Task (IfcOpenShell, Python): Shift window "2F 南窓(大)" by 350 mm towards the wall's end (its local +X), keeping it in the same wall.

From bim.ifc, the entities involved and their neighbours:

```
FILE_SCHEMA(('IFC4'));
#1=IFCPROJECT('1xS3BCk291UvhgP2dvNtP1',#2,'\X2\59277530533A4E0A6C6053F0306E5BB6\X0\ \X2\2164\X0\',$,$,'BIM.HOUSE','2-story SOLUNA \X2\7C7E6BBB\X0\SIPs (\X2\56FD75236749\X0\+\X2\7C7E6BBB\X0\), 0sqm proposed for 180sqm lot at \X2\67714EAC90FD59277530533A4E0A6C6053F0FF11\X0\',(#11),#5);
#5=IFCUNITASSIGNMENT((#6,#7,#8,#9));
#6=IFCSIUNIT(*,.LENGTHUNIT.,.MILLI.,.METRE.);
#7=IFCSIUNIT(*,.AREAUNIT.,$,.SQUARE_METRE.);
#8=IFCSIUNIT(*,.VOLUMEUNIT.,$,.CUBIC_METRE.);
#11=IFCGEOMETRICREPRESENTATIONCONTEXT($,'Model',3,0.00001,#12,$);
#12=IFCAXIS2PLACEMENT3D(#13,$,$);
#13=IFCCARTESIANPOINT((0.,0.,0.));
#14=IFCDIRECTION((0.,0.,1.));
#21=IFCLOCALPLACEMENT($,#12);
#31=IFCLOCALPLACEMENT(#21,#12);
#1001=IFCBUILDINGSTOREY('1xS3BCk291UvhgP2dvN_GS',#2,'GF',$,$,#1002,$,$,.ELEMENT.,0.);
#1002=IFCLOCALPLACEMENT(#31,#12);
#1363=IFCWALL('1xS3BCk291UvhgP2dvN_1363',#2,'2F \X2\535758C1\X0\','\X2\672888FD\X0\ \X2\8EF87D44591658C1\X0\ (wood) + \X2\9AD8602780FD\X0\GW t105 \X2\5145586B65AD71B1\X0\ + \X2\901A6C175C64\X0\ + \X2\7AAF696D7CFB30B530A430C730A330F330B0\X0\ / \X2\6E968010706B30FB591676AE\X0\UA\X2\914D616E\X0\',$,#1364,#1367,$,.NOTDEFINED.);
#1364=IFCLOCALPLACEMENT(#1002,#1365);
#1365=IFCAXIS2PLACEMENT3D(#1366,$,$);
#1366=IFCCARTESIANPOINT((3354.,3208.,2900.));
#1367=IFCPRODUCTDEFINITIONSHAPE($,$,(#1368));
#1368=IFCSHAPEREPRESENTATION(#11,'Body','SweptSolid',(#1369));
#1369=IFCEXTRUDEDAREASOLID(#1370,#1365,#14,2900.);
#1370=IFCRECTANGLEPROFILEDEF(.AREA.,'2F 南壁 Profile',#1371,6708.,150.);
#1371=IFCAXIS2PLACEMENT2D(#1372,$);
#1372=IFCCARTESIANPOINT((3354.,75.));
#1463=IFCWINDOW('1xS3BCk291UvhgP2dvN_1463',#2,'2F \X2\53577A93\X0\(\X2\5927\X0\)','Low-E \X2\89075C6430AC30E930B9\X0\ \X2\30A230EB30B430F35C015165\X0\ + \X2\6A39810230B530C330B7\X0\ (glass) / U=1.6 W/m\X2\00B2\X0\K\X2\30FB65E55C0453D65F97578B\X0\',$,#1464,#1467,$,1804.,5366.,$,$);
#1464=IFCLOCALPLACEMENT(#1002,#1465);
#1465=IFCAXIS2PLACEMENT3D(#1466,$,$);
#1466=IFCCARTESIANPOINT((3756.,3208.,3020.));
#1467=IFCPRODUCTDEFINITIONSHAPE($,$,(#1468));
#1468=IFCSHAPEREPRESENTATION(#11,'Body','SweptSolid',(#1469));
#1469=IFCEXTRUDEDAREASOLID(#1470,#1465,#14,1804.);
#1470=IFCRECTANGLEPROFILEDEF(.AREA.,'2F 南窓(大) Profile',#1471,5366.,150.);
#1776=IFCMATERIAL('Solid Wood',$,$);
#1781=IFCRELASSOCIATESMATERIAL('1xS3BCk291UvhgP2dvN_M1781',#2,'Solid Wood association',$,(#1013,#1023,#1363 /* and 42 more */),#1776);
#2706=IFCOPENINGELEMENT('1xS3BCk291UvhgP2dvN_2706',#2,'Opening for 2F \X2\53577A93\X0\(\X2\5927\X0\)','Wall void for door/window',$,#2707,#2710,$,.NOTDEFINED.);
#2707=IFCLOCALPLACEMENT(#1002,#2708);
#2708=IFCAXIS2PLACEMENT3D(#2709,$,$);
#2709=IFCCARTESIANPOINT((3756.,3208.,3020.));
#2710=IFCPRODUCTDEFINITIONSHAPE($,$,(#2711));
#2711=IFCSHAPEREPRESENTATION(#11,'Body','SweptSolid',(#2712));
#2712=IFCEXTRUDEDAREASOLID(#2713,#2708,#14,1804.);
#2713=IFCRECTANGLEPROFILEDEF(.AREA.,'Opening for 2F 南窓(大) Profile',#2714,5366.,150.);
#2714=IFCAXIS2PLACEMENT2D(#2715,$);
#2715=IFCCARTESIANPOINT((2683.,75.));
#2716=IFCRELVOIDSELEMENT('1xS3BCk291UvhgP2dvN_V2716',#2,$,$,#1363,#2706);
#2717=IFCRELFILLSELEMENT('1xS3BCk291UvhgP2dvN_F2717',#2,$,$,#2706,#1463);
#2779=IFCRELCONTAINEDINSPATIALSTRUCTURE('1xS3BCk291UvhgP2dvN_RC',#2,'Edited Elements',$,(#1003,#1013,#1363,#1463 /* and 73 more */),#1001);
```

```python
import ifcopenshell
import ifcopenshell.api.geometry
import ifcopenshell.util.placement
import ifcopenshell.util.unit

model = ifcopenshell.open("bim.ifc")
unit_scale = ifcopenshell.util.unit.calculate_unit_scale(model)

window = model.by_guid("1xS3BCk291UvhgP2dvN_1463")
opening = window.FillsVoids[0].RelatingOpeningElement
wall = opening.VoidsElements[0].RelatingBuildingElement

wall_matrix = ifcopenshell.util.placement.get_local_placement(wall.ObjectPlacement)
shift = wall_matrix[:3, 0] * 0.35 / unit_scale
before = ifcopenshell.util.placement.get_local_placement(window.ObjectPlacement)[:3, 3].copy()

# The window is not placed relative to its opening, so move both.
for product in (opening, window):
    matrix = ifcopenshell.util.placement.get_local_placement(product.ObjectPlacement)
    matrix[:3, 3] += shift
    ifcopenshell.api.geometry.edit_object_placement(model, product=product, matrix=matrix, is_si=False)

after = ifcopenshell.util.placement.get_local_placement(window.ObjectPlacement)[:3, 3]
print("window moved by", (after - before).round(3) + 0.0)

model.write("bim_updated.ifc")
```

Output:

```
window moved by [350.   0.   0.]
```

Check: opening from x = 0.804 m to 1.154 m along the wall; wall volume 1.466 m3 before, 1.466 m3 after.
